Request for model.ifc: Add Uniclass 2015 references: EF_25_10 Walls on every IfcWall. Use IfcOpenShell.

First a look at what the model holds.

```python
import ifcopenshell

model = ifcopenshell.open("model.ifc")
print(model.schema)
print("classifications:", [c.Name for c in model.by_type("IfcClassification")])
for ifc_class in ("IfcDoor", "IfcRoof", "IfcStair", "IfcWall", "IfcWindow"):
    print(ifc_class, len(model.by_type(ifc_class)))
```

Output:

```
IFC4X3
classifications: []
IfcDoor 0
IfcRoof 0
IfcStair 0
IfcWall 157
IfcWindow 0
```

```python
import ifcopenshell
import ifcopenshell.api.classification

model = ifcopenshell.open("model.ifc")

system = ifcopenshell.api.classification.add_classification(model, classification="Uniclass 2015")

codes = {
    "IfcWall": ("EF_25_10", "Walls"),
}
for ifc_class, (code, name) in codes.items():
    products = model.by_type(ifc_class)
    ifcopenshell.api.classification.add_reference(
        model, products=products, classification=system, identification=code, name=name
    )
    print(code, len(products))

model.write("model_rev.ifc")
```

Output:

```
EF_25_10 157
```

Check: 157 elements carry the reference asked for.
